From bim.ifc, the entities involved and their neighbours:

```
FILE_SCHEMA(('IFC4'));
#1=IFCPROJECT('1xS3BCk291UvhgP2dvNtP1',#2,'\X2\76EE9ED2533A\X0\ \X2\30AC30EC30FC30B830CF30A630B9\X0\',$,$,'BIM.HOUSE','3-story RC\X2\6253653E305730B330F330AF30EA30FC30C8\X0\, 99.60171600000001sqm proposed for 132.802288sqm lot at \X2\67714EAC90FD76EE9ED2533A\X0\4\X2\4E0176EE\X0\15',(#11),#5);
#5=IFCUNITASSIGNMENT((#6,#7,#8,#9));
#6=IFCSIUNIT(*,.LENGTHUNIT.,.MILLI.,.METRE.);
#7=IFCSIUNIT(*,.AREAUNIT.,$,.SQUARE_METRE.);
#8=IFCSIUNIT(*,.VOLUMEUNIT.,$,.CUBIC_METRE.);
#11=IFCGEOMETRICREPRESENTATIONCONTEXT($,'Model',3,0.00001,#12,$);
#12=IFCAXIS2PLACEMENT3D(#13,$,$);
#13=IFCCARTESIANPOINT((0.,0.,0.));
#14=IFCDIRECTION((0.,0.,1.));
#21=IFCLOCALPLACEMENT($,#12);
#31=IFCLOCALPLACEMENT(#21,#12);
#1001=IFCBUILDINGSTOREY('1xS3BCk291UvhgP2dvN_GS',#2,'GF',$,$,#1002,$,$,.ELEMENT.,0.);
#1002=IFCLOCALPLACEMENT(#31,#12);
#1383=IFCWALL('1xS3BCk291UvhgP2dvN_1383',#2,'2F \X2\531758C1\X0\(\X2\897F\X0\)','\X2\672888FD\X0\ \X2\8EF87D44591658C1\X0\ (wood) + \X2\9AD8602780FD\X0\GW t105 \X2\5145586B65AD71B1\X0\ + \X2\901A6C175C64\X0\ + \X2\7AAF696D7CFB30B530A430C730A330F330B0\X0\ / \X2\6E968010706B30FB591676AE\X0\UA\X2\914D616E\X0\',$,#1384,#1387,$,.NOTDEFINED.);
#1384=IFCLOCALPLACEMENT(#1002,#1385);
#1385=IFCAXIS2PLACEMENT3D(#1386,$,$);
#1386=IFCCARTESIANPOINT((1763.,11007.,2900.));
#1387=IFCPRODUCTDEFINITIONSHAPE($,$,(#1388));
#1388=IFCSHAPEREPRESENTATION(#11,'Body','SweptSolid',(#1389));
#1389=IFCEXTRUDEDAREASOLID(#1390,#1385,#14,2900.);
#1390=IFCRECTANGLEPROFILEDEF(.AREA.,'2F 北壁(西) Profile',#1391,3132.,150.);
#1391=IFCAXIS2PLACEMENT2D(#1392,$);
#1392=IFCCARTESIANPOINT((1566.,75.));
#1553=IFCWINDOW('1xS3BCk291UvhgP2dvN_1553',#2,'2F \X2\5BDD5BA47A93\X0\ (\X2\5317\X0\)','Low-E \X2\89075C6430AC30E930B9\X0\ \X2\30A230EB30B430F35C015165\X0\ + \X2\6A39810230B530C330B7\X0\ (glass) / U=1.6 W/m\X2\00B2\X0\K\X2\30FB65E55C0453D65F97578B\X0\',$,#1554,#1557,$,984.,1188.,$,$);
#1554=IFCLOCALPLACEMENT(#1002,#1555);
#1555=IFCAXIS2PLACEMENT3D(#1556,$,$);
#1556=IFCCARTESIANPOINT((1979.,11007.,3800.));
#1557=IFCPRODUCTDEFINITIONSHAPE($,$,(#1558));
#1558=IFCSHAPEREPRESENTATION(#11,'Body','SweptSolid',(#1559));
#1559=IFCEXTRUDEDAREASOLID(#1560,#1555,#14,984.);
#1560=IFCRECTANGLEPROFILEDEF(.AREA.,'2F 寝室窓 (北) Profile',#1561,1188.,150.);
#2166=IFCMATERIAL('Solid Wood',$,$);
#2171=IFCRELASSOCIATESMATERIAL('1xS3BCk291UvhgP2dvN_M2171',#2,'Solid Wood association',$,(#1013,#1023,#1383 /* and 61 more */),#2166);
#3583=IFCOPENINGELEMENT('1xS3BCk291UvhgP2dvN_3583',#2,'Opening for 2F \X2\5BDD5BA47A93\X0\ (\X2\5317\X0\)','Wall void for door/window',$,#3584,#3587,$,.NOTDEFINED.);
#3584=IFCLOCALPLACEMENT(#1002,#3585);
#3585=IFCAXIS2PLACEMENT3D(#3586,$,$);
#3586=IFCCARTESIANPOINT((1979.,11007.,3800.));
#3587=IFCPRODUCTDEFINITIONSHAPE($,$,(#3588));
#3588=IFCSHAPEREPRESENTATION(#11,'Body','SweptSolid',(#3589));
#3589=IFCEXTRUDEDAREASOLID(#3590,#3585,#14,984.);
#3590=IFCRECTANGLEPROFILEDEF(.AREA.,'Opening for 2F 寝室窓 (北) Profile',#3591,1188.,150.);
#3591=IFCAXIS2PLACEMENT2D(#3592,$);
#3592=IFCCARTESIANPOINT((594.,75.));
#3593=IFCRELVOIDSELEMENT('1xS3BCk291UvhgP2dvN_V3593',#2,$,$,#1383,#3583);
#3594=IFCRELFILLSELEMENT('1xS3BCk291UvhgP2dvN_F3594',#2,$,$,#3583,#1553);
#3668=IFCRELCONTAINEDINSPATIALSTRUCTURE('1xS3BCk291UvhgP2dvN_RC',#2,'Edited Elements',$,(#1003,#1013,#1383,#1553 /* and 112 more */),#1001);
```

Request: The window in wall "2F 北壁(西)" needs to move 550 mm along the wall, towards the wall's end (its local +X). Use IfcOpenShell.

```python
import ifcopenshell
import ifcopenshell.api.geometry
import ifcopenshell.util.placement

model = ifcopenshell.open("bim.ifc")

window = model.by_guid("1xS3BCk291UvhgP2dvN_1553")
opening = window.FillsVoids[0].RelatingOpeningElement
wall = opening.VoidsElements[0].RelatingBuildingElement

wall_matrix = ifcopenshell.util.placement.get_local_placement(wall.ObjectPlacement)
shift = wall_matrix[:3, 0] * 550.0
before = ifcopenshell.util.placement.get_local_placement(window.ObjectPlacement)[:3, 3].copy()

# The window is not placed relative to its opening, so move both.
for product in (opening, window):
    matrix = ifcopenshell.util.placement.get_local_placement(product.ObjectPlacement)
    matrix[:3, 3] += shift
    ifcopenshell.api.geometry.edit_object_placement(model, product=product, matrix=matrix, is_si=False)

after = ifcopenshell.util.placement.get_local_placement(window.ObjectPlacement)[:3, 3]
print("window moved by", (after - before).round(3) + 0.0)

model.write("bim_rev.ifc")
```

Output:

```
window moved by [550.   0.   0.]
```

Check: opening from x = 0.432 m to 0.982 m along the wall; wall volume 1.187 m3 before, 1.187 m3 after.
